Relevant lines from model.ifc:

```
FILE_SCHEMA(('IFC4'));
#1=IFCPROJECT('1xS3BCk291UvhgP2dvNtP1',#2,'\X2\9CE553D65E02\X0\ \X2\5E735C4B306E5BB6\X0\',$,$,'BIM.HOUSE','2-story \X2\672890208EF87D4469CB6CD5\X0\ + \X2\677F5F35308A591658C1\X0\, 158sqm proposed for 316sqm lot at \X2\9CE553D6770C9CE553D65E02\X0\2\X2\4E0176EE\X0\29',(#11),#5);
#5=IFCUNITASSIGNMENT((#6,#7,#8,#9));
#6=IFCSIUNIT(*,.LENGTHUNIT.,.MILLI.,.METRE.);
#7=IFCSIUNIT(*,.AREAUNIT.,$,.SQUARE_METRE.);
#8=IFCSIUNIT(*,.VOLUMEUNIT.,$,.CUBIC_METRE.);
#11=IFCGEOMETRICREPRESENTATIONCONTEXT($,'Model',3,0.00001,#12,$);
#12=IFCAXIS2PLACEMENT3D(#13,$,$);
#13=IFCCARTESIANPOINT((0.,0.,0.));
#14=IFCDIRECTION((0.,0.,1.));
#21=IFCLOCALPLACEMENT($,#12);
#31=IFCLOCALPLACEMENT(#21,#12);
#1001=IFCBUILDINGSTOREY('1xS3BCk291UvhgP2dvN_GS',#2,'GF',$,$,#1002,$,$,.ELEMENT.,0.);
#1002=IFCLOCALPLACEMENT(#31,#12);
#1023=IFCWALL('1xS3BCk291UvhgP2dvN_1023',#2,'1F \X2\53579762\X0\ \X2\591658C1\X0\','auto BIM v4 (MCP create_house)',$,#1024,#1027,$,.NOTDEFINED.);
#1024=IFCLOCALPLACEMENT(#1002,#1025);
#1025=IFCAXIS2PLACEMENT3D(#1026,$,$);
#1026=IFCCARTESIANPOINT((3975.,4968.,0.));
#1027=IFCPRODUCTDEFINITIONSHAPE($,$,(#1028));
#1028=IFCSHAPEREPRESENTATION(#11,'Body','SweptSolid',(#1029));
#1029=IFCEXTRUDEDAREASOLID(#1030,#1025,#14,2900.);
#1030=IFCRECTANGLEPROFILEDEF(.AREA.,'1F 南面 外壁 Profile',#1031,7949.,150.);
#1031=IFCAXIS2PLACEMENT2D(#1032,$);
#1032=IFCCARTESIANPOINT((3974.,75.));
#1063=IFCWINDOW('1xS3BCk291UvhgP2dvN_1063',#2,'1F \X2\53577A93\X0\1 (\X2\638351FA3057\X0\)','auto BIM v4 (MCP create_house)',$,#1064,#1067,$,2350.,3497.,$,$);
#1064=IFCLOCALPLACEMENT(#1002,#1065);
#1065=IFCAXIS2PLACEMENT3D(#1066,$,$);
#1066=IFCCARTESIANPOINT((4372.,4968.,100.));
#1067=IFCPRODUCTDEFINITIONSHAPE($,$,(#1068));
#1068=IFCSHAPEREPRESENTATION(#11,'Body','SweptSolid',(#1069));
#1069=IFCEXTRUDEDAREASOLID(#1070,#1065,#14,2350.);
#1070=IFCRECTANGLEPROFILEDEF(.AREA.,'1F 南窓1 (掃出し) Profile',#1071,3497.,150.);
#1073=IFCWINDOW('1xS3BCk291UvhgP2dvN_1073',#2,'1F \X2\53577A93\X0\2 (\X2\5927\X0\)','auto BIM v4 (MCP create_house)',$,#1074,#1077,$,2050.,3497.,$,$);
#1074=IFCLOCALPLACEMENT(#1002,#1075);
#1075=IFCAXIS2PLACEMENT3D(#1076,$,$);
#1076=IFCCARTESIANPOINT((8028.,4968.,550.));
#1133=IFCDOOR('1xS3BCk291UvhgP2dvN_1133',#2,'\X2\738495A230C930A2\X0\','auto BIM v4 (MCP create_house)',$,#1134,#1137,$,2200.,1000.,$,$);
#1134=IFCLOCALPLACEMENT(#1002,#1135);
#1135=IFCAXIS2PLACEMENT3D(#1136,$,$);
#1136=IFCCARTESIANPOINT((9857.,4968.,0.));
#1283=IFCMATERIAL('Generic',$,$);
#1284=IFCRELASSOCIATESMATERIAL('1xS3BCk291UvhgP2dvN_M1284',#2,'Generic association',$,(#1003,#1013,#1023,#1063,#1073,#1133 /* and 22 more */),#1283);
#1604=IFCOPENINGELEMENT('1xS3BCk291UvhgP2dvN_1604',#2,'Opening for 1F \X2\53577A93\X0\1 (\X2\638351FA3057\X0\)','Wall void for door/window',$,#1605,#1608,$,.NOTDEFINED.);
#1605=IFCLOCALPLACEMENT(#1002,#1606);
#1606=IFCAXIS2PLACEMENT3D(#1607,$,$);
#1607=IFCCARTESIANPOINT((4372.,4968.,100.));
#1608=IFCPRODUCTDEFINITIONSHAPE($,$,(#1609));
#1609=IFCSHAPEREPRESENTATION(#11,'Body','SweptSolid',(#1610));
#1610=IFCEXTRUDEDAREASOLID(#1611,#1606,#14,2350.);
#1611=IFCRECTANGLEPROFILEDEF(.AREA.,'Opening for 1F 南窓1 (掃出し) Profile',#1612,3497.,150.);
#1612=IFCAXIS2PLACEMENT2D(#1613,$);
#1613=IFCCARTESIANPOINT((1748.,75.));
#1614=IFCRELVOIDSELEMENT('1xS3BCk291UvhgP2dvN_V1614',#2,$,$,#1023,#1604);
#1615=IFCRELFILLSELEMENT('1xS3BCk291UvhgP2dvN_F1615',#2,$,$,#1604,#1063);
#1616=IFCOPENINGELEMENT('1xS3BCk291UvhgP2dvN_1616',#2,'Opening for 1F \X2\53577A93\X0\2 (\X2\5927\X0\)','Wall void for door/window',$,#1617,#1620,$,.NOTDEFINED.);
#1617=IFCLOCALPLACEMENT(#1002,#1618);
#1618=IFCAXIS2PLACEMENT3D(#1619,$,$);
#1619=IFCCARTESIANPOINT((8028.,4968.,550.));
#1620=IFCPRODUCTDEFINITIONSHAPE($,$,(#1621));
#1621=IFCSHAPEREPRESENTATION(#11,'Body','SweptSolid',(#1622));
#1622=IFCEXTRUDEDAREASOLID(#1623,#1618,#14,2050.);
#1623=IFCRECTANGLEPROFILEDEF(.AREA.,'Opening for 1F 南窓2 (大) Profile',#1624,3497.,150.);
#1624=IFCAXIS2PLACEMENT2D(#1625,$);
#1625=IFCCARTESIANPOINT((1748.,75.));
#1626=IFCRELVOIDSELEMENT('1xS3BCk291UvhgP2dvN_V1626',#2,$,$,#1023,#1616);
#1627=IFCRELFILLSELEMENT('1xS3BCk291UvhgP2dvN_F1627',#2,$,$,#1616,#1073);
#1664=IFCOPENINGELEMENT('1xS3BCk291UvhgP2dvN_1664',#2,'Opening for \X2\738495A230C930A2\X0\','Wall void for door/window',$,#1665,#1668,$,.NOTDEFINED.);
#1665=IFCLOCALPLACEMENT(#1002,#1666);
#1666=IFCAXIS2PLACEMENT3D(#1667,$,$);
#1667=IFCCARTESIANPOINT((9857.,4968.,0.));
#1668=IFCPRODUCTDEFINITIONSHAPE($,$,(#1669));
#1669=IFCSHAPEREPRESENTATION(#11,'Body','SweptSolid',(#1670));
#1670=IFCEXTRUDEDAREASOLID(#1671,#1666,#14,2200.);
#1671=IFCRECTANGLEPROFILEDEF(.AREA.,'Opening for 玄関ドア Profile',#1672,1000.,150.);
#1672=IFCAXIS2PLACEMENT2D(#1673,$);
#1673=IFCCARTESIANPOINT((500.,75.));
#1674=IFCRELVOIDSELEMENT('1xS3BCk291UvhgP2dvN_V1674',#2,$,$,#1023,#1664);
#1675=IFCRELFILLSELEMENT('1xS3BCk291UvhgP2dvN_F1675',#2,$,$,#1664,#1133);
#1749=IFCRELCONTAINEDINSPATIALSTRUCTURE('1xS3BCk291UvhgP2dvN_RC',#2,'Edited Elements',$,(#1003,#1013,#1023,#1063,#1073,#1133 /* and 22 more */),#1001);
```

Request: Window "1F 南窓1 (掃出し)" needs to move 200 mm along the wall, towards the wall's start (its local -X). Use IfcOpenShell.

```python
import ifcopenshell
import ifcopenshell.api.geometry
import ifcopenshell.util.placement
import ifcopenshell.util.unit

model = ifcopenshell.open("model.ifc")
unit_scale = ifcopenshell.util.unit.calculate_unit_scale(model)

window = model.by_id(1063)
opening = window.FillsVoids[0].RelatingOpeningElement
wall = opening.VoidsElements[0].RelatingBuildingElement

wall_matrix = ifcopenshell.util.placement.get_local_placement(wall.ObjectPlacement)
shift = wall_matrix[:3, 0] * -0.2 / unit_scale
before = ifcopenshell.util.placement.get_local_placement(window.ObjectPlacement)[:3, 3].copy()

# The window is not placed relative to its opening, so move both.
for product in (opening, window):
    matrix = ifcopenshell.util.placement.get_local_placement(product.ObjectPlacement)
    matrix[:3, 3] += shift
    ifcopenshell.api.geometry.edit_object_placement(model, product=product, matrix=matrix, is_si=False)

after = ifcopenshell.util.placement.get_local_placement(window.ObjectPlacement)[:3, 3]
print("window moved by", (after - before).round(3) + 0.0)

model.write("model_edited.ifc")
```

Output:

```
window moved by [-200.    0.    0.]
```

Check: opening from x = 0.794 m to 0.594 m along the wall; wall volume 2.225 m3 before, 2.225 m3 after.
